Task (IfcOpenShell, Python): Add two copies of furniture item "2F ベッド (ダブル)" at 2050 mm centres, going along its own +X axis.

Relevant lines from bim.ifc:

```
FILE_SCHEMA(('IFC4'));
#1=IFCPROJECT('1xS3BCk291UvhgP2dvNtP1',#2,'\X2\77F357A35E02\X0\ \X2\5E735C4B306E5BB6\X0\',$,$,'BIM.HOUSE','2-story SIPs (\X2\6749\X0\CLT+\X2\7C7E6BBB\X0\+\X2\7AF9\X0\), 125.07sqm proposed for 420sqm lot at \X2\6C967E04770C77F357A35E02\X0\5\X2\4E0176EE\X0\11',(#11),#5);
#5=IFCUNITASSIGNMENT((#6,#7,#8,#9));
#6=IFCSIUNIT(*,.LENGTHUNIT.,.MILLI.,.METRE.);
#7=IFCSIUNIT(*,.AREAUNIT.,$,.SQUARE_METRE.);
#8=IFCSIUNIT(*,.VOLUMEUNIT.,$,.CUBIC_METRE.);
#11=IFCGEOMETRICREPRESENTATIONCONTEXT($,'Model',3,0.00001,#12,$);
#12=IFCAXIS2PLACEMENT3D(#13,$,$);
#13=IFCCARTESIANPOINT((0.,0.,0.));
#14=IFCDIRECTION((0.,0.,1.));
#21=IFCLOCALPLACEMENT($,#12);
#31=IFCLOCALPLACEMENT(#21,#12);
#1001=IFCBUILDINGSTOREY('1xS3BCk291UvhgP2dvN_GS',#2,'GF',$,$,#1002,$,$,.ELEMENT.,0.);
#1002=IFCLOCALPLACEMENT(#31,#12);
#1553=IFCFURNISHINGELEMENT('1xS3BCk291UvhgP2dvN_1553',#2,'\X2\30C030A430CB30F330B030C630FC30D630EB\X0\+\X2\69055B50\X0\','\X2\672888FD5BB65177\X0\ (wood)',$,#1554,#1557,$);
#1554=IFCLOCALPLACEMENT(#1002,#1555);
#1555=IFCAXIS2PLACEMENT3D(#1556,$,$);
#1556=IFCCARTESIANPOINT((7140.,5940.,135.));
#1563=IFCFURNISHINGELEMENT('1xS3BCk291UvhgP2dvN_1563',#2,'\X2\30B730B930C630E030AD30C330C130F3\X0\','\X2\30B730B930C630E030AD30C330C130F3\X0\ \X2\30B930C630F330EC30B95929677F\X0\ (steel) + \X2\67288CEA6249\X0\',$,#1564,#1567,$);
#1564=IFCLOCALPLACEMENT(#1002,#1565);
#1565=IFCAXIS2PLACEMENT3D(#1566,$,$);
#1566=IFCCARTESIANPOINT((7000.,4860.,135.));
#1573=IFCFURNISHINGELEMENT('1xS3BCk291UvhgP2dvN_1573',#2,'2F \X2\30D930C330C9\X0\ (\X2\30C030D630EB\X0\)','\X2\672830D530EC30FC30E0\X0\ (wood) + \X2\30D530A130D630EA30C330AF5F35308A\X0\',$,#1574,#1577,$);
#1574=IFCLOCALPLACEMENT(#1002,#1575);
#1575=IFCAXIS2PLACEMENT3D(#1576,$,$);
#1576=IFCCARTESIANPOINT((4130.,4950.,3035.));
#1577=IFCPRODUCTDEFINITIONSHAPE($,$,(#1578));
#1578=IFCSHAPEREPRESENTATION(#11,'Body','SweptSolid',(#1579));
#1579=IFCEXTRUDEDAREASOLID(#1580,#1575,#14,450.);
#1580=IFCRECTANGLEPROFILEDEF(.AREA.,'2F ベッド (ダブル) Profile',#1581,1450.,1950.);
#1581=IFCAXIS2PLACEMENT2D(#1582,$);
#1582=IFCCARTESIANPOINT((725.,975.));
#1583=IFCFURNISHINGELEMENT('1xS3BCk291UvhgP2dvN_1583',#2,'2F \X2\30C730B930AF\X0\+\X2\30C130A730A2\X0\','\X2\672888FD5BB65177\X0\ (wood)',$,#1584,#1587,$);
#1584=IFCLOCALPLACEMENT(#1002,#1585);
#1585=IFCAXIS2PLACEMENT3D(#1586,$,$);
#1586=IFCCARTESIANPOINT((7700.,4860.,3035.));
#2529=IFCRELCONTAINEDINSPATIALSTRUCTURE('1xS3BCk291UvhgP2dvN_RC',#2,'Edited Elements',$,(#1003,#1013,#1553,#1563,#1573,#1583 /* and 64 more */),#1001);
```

```python
import ifcopenshell
import ifcopenshell.api.geometry
import ifcopenshell.api.root
import ifcopenshell.util.element
import ifcopenshell.util.placement
import ifcopenshell.util.unit

model = ifcopenshell.open("bim.ifc")
unit_scale = ifcopenshell.util.unit.calculate_unit_scale(model)


def reuse_history(source, copy):
    """copy_class also copies each property set's owner history, people and application; keep the originals."""
    for rel in copy.IsDefinedBy:
        if rel.is_a("IfcRelDefinesByProperties") and (history := rel.RelatingPropertyDefinition.OwnerHistory):
            rel.RelatingPropertyDefinition.OwnerHistory = source.OwnerHistory
            ifcopenshell.util.element.remove_deep2(model, history)


source = model.by_id(1573)
base = ifcopenshell.util.placement.get_local_placement(source.ObjectPlacement)
step = base[:3, 0] * 2.05 / unit_scale

for i in range(1, 3):
    copy = ifcopenshell.api.root.copy_class(model, product=source)
    copy.Representation = ifcopenshell.util.element.copy_deep(
        model, source.Representation, exclude=["IfcGeometricRepresentationContext", "IfcRepresentationMap"]
    )
    reuse_history(source, copy)
    matrix = base.copy()
    matrix[:3, 3] += i * step
    print("added at", matrix[:3, 3].round(3) + 0.0)
    ifcopenshell.api.geometry.edit_object_placement(model, product=copy, matrix=matrix, is_si=False)

model.write("bim-out.ifc")
```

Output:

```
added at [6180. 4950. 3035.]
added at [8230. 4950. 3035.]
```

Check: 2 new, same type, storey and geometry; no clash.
